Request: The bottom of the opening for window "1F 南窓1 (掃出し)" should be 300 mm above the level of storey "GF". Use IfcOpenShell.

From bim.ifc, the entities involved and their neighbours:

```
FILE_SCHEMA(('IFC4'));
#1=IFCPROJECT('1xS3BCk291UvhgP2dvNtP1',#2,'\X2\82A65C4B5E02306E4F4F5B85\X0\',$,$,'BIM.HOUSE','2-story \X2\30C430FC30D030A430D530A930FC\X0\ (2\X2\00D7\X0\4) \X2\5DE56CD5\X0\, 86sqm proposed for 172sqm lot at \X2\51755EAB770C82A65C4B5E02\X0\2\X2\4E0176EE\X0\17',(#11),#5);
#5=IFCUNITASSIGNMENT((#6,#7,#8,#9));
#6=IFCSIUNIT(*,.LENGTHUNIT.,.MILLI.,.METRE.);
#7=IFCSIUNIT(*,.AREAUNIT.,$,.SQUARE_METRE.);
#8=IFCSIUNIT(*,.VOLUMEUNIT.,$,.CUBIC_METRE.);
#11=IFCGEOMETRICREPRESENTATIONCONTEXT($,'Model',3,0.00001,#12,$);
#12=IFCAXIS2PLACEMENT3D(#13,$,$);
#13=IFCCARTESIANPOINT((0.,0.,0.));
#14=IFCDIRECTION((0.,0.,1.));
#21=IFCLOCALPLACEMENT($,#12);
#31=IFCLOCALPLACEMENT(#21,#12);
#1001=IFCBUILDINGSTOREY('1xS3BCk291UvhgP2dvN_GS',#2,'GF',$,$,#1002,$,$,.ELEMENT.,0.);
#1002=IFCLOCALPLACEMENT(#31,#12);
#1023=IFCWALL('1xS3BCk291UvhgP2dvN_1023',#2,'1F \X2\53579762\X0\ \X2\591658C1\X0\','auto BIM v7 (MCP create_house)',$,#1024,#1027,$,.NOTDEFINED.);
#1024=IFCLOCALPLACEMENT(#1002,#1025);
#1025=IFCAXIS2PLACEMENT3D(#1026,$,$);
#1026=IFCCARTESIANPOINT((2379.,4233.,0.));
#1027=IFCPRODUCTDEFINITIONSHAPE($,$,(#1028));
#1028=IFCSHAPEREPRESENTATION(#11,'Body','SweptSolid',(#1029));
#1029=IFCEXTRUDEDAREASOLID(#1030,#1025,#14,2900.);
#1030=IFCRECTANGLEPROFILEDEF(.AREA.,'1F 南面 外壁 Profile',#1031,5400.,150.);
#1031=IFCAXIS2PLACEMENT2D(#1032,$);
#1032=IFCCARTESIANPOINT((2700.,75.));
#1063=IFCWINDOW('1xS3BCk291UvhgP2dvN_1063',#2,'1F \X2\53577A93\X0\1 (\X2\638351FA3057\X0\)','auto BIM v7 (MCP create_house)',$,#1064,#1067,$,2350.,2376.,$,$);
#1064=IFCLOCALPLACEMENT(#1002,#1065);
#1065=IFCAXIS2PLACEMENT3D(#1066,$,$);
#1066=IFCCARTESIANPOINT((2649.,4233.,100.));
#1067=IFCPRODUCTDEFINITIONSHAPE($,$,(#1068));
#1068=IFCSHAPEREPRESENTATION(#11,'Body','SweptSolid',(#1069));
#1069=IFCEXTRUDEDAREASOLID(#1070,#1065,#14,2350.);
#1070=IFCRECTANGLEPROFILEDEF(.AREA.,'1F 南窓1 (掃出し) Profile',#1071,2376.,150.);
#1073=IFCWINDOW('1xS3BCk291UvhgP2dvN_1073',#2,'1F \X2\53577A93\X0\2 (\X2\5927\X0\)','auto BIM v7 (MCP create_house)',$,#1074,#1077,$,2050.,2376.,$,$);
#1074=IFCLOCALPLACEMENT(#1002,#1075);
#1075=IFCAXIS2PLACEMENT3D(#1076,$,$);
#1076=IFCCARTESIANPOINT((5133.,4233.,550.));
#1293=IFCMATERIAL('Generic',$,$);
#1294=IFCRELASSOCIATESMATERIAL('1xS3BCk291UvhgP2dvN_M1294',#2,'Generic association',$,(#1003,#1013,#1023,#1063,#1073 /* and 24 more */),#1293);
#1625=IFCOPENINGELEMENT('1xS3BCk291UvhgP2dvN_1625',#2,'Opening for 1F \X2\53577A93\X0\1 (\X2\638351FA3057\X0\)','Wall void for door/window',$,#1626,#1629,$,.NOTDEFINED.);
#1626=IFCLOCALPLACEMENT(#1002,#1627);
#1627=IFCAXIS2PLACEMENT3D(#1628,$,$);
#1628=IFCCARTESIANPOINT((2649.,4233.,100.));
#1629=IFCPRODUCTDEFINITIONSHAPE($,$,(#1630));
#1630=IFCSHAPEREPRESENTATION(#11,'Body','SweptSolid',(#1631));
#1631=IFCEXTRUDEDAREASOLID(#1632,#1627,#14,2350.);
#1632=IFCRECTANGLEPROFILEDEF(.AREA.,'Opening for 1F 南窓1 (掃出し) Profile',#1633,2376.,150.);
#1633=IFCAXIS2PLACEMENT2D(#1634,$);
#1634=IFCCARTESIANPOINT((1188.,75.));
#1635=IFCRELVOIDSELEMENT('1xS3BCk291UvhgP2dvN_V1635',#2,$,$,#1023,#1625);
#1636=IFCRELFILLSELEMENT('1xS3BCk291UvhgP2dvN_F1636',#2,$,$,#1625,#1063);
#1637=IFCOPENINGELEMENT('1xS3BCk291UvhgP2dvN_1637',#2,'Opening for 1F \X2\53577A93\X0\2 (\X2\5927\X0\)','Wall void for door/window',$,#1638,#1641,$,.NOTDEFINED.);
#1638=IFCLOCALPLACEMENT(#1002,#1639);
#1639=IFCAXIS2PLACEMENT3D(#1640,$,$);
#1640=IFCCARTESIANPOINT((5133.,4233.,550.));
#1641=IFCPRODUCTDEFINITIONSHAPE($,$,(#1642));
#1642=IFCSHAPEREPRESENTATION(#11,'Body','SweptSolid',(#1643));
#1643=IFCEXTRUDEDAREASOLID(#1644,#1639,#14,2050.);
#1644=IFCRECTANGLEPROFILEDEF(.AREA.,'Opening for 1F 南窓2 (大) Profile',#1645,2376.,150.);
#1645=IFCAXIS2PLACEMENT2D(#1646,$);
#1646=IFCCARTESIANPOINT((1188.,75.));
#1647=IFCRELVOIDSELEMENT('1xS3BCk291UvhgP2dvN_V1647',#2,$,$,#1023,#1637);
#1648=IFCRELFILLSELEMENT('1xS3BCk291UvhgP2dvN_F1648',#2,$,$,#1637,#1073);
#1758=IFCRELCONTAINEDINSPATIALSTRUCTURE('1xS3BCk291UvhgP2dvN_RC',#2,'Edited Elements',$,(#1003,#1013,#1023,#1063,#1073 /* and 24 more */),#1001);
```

```python
import numpy as np
import ifcopenshell
import ifcopenshell.api.geometry
import ifcopenshell.geom
import ifcopenshell.util.element
import ifcopenshell.util.placement
import ifcopenshell.util.shape
import ifcopenshell.util.unit

model = ifcopenshell.open("bim.ifc")
unit_scale = ifcopenshell.util.unit.calculate_unit_scale(model)

window = model.by_guid("1xS3BCk291UvhgP2dvN_1063")
opening = window.FillsVoids[0].RelatingOpeningElement
storey = ifcopenshell.util.element.get_container(window, ifc_class="IfcBuildingStorey")
level = ifcopenshell.util.placement.get_local_placement(storey.ObjectPlacement)[2, 3]

# The opening's origin need not be at the sill, so measure its lowest point.
shape = ifcopenshell.geom.create_shape(ifcopenshell.geom.settings(), opening)
bottom = ifcopenshell.util.shape.get_shape_bottom_elevation(shape, shape.geometry) / unit_scale
dz = level + 300.0 - bottom

shift = np.array([0.0, 0.0, dz])
# The window is not placed relative to its opening, so move both.
for product in (opening, window):
    matrix = ifcopenshell.util.placement.get_local_placement(product.ObjectPlacement)
    matrix[:3, 3] += shift
    ifcopenshell.api.geometry.edit_object_placement(model, product=product, matrix=matrix, is_si=False)

print(f"moved by {dz * unit_scale:+.3f} m")

model.write("bim-out.ifc")
```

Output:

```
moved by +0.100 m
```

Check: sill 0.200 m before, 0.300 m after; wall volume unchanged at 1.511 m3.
